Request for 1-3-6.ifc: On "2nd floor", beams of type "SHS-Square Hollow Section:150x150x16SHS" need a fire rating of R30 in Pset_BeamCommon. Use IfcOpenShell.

First a look at what the model holds.

```python
import ifcopenshell
import ifcopenshell.util.element

model = ifcopenshell.open("1-3-6.ifc")
print(model.schema)
storey = next(s for s in model.by_type("IfcBuildingStorey") if s.Name == "2nd floor")
beams = [e for e in ifcopenshell.util.element.get_decomposition(storey) if e.is_a("IfcBeam")]
seen = {}
for e in beams:
    element_type = ifcopenshell.util.element.get_type(e)
    key = (element_type.Name if element_type != e and element_type else None, ifcopenshell.util.element.get_pset(e, "Pset_BeamCommon", "FireRating"))
    seen[key] = seen.get(key, 0) + 1
for (name, value), count in sorted(seen.items(), key=str):
    print(count, "x", name, "|", value)
```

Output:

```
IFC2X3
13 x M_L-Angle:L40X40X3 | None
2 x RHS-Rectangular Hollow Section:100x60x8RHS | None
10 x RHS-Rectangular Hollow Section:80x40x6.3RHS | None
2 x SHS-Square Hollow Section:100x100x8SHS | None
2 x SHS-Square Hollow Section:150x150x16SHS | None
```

```python
import ifcopenshell
import ifcopenshell.api.pset
import ifcopenshell.util.element

model = ifcopenshell.open("1-3-6.ifc")

storey = next(s for s in model.by_type("IfcBuildingStorey") if s.Name == "2nd floor")
beams = [e for e in ifcopenshell.util.element.get_decomposition(storey) if e.is_a("IfcBeam")]

count = 0
for e in beams:
    element_type = ifcopenshell.util.element.get_type(e)
    if element_type in (None, e) or element_type.Name != "SHS-Square Hollow Section:150x150x16SHS":
        continue
    # add_pset returns the element's existing set when there is one.
    pset = ifcopenshell.api.pset.add_pset(model, product=e, name="Pset_BeamCommon")
    ifcopenshell.api.pset.edit_pset(model, pset=pset, properties={"FireRating": "R30"})
    count += 1

print(count, "beams updated")

model.write("1-3-6-out.ifc")
```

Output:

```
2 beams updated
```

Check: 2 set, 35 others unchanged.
